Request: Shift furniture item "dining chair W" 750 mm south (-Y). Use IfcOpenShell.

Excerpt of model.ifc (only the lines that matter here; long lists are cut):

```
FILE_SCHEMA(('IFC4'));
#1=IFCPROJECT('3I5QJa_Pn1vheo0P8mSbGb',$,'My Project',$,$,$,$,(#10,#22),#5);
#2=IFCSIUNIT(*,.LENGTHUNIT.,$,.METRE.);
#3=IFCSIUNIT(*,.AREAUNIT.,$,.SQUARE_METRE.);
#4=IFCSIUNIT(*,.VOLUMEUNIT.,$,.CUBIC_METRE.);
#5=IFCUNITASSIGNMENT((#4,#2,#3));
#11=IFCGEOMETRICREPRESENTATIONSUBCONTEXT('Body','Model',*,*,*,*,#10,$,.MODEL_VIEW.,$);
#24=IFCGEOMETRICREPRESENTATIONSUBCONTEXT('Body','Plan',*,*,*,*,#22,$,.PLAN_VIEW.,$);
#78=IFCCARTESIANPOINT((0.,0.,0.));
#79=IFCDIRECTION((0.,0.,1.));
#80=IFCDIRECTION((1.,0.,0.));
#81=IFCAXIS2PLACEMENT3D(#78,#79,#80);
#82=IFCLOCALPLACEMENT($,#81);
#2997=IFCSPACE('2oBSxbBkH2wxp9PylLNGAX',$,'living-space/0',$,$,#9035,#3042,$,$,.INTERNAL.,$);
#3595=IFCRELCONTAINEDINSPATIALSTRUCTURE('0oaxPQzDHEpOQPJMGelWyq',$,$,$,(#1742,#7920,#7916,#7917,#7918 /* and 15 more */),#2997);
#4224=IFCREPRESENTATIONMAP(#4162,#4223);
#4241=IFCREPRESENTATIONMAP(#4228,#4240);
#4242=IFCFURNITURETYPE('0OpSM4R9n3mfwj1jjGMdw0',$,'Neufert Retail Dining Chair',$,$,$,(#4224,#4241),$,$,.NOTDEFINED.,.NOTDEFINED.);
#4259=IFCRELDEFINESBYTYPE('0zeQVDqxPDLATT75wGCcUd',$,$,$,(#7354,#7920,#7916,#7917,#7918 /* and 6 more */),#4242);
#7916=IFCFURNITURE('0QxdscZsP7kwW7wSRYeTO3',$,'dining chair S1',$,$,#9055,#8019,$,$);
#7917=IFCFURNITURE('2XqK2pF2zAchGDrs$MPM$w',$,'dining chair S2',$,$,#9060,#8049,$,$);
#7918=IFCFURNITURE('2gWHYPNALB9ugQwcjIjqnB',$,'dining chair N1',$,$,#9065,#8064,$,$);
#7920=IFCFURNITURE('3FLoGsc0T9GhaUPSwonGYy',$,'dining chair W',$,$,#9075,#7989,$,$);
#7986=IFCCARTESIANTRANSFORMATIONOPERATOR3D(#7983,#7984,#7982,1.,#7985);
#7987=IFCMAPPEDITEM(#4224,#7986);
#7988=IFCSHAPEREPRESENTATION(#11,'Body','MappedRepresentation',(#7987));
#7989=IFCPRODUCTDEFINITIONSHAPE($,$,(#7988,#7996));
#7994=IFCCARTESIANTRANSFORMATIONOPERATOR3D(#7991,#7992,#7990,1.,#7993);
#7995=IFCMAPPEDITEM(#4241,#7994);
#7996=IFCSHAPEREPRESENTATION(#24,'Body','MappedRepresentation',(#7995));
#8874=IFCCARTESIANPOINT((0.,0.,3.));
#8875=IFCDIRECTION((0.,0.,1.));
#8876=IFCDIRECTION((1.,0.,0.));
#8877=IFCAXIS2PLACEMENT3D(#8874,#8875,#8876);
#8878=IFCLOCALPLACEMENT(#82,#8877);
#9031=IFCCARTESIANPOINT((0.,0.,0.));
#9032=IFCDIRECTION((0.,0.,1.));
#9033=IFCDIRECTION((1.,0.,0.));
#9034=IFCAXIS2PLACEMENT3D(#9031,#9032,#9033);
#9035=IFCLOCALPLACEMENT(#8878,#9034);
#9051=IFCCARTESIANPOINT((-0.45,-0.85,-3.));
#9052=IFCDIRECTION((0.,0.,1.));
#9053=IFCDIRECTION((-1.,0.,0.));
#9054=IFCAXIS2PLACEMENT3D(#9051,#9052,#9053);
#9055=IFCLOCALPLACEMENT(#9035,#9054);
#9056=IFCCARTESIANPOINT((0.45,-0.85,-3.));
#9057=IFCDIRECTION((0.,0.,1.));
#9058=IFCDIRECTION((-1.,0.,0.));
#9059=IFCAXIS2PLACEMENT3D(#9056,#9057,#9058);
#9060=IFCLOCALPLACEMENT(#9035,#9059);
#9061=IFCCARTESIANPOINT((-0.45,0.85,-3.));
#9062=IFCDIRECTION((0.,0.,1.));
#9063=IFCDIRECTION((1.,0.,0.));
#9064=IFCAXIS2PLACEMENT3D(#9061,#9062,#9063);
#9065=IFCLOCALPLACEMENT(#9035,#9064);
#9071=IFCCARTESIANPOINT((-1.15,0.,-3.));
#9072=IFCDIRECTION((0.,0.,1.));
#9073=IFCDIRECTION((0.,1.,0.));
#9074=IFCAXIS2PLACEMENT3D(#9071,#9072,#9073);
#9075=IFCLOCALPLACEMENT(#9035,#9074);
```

```python
import ifcopenshell
import ifcopenshell.api.geometry
import ifcopenshell.util.placement
import ifcopenshell.util.unit

model = ifcopenshell.open("model.ifc")
unit_scale = ifcopenshell.util.unit.calculate_unit_scale(model)

item = model.by_id(7920)
matrix = ifcopenshell.util.placement.get_local_placement(item.ObjectPlacement)
matrix[1, 3] -= 0.75 / unit_scale
ifcopenshell.api.geometry.edit_object_placement(model, product=item, matrix=matrix, is_si=False)

print(ifcopenshell.util.placement.get_local_placement(item.ObjectPlacement).round(3) + 0.0)

model.write("model_v2.ifc")
```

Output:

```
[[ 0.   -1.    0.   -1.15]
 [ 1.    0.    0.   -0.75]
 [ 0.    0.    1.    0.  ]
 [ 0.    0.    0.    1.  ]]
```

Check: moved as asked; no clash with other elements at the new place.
